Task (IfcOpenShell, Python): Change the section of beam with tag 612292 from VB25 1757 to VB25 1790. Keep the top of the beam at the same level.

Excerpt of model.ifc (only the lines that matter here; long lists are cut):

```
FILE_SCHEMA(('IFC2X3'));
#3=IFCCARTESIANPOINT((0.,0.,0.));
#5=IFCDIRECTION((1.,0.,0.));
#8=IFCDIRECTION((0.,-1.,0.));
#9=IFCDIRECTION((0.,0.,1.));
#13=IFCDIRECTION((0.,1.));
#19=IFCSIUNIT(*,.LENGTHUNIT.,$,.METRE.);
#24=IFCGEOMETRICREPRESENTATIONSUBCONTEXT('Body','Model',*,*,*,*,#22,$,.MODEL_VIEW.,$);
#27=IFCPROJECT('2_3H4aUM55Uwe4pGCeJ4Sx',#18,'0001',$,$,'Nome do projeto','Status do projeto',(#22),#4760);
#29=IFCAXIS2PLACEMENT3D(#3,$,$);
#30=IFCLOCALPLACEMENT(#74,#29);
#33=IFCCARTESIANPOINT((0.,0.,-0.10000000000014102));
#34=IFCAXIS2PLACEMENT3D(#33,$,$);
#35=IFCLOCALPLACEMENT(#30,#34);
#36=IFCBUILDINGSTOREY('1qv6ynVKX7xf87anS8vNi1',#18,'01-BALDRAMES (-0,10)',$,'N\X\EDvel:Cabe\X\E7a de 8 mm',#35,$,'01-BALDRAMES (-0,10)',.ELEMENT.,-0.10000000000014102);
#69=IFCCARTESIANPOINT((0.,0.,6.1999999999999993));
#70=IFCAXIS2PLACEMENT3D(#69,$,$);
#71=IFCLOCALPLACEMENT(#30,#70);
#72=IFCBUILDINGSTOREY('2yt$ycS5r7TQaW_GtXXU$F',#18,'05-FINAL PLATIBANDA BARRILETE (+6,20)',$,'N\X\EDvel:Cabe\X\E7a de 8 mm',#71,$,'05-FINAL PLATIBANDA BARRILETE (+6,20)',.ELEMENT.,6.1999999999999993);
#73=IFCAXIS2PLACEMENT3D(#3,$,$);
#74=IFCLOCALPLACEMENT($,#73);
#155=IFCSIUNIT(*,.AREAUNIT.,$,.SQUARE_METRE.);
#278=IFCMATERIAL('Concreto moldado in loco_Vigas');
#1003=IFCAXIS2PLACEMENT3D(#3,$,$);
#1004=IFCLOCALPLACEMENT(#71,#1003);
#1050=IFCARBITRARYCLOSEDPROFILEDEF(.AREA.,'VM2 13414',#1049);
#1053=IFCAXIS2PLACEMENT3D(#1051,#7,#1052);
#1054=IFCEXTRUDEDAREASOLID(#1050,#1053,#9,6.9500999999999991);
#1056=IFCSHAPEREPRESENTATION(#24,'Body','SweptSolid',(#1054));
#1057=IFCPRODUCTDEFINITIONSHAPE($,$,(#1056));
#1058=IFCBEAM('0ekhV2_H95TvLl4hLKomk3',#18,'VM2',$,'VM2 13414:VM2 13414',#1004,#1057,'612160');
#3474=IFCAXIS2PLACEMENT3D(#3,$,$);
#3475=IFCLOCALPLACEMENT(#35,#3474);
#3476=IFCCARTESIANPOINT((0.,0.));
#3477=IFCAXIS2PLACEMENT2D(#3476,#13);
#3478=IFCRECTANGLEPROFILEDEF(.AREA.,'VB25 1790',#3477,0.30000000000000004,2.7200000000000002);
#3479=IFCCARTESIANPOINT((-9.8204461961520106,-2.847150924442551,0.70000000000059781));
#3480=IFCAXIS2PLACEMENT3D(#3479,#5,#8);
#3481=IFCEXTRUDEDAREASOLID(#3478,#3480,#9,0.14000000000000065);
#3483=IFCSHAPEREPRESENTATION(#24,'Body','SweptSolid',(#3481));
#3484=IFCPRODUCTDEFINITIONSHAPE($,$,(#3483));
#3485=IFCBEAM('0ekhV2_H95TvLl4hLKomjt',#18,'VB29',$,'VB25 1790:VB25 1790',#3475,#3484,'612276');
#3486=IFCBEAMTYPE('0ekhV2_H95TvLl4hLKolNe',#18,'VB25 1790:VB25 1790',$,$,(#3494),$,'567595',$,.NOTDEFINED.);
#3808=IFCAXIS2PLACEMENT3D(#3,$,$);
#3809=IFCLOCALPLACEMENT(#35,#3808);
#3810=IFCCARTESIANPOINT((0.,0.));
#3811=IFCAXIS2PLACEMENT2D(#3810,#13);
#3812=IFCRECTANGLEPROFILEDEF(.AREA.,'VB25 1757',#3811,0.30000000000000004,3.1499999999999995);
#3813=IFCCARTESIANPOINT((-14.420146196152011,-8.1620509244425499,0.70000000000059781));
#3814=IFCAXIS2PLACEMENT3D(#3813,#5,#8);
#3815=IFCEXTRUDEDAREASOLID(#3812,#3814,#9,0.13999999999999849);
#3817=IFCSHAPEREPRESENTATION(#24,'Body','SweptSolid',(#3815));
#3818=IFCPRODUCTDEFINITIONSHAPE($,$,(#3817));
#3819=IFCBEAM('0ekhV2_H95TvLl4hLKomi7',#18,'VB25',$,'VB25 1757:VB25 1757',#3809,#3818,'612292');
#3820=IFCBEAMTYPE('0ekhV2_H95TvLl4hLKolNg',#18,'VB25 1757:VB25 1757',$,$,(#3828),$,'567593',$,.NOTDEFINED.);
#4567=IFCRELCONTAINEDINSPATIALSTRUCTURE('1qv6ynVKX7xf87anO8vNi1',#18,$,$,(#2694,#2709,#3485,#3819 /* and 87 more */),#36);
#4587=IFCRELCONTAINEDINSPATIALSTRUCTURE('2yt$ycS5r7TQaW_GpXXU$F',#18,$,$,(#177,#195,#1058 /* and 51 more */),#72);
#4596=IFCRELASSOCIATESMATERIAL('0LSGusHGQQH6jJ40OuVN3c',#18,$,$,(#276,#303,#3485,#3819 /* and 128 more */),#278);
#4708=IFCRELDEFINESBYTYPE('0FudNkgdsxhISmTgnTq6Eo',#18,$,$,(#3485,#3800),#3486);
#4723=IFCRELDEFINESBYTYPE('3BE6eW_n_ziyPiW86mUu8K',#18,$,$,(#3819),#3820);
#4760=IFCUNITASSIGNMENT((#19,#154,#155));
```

```python
import ifcopenshell
import ifcopenshell.api.type
import ifcopenshell.util.element
import ifcopenshell.util.representation

model = ifcopenshell.open("model.ifc")

member = model.by_guid("0ekhV2_H95TvLl4hLKomi7")
source = next(p for p in model.by_type("IfcRectangleProfileDef") if p.ProfileName == "VB25 1790")

body = ifcopenshell.util.representation.get_representation(member, "Model", "Body")
solid = body.Items[0]
old_profile = solid.SweptArea

# Copy the section's sizes but keep this member's own profile position.
profile = ifcopenshell.util.element.copy(model, source)
# Profiles are centred, so shift by half the change in depth to hold the top.
shift = (old_profile.XDim - profile.XDim) / 2
x, y = old_profile.Position.Location.Coordinates
up = (0.0, -1.0)  # upwards, in the solid's own plane
location = model.createIfcCartesianPoint((x + up[0] * shift, y + up[1] * shift))
profile.Position = model.createIfcAxis2Placement2D(location, old_profile.Position.RefDirection)
solid.SweptArea = profile
if not model.get_total_inverses(old_profile):
    ifcopenshell.util.element.remove_deep2(model, old_profile)

new_type = model.by_id(3486)
ifcopenshell.api.type.assign_type(
    model, related_objects=[member], relating_type=new_type, should_map_representations=False
)
member.ObjectType = "VB25 1790:VB25 1790"

print(solid.SweptArea)

model.write("model-out.ifc")
```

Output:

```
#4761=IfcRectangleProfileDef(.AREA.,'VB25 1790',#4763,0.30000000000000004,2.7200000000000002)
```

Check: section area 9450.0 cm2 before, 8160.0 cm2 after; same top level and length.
